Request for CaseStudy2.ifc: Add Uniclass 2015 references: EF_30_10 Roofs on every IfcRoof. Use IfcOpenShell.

First a look at what the model holds.

```python
import ifcopenshell

model = ifcopenshell.open("CaseStudy2.ifc")
print(model.schema)
print("classifications:", [c.Name for c in model.by_type("IfcClassification")])
for ifc_class in ("IfcDoor", "IfcRoof", "IfcStair", "IfcWall", "IfcWindow"):
    print(ifc_class, len(model.by_type(ifc_class)))
```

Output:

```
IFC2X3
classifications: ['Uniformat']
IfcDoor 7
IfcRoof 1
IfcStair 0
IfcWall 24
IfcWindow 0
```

```python
import ifcopenshell
import ifcopenshell.api.classification

model = ifcopenshell.open("CaseStudy2.ifc")

# IFC2X3 requires Source and Edition and has no link from the project to the system.
system = model.create_entity("IfcClassification", Source="NBS", Edition="2015", Name="Uniclass 2015")

codes = {
    "IfcRoof": ("EF_30_10", "Roofs"),
}
for ifc_class, (code, name) in codes.items():
    products = model.by_type(ifc_class)
    ifcopenshell.api.classification.add_reference(
        model, products=products, classification=system, identification=code, name=name
    )
    print(code, len(products))

model.write("CaseStudy2_updated.ifc")
```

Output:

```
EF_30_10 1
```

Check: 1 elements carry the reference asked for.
